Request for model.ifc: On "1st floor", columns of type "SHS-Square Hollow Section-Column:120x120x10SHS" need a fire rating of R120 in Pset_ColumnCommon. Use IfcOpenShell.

First a look at what the model holds.

```python
import ifcopenshell
import ifcopenshell.util.element

model = ifcopenshell.open("model.ifc")
print(model.schema)
storey = next(s for s in model.by_type("IfcBuildingStorey") if s.Name == "1st floor")
columns = [e for e in ifcopenshell.util.element.get_decomposition(storey) if e.is_a("IfcColumn")]
seen = {}
for e in columns:
    element_type = ifcopenshell.util.element.get_type(e)
    key = (element_type.Name if element_type != e and element_type else None, ifcopenshell.util.element.get_pset(e, "Pset_ColumnCommon", "FireRating"))
    seen[key] = seen.get(key, 0) + 1
for (name, value), count in sorted(seen.items(), key=str):
    print(count, "x", name, "|", value)
```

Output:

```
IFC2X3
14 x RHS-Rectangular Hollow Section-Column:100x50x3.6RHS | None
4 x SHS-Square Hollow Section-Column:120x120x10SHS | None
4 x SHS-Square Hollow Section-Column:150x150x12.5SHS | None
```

```python
import ifcopenshell
import ifcopenshell.api.pset
import ifcopenshell.util.element

model = ifcopenshell.open("model.ifc")

storey = next(s for s in model.by_type("IfcBuildingStorey") if s.Name == "1st floor")
columns = [e for e in ifcopenshell.util.element.get_decomposition(storey) if e.is_a("IfcColumn")]

count = 0
for e in columns:
    element_type = ifcopenshell.util.element.get_type(e)
    if element_type in (None, e) or element_type.Name != "SHS-Square Hollow Section-Column:120x120x10SHS":
        continue
    # add_pset returns the element's existing set when there is one.
    pset = ifcopenshell.api.pset.add_pset(model, product=e, name="Pset_ColumnCommon")
    ifcopenshell.api.pset.edit_pset(model, pset=pset, properties={"FireRating": "R120"})
    count += 1

print(count, "columns updated")

model.write("model_rev.ifc")
```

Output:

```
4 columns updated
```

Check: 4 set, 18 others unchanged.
